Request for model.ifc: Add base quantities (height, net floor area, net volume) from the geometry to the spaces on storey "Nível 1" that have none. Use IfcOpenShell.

First a look at what the model holds.

```python
import ifcopenshell
import ifcopenshell.util.element
import ifcopenshell.util.unit

model = ifcopenshell.open("model.ifc")
print(model.schema)
for unit_type in ("LENGTHUNIT", "AREAUNIT", "VOLUMEUNIT"):
    print(unit_type, ifcopenshell.util.unit.calculate_unit_scale(model, unit_type))
storey = next(s for s in model.by_type("IfcBuildingStorey") if s.Name == "Nível 1")
spaces = [e for e in ifcopenshell.util.element.get_decomposition(storey) if e.is_a("IfcSpace")]
for e in sorted(spaces, key=lambda e: e.id()):
    print(e.id(), e.is_a(), e.Name, list(ifcopenshell.util.element.get_psets(e, qtos_only=True)), sep=" | ")
```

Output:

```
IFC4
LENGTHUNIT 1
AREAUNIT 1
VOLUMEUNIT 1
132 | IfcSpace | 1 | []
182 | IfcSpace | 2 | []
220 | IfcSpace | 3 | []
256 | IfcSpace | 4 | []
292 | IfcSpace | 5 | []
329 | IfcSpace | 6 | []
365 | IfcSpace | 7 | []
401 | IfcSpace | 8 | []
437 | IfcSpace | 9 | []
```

```python
import ifcopenshell
import ifcopenshell.api.pset
import ifcopenshell.geom
import ifcopenshell.util.element
import ifcopenshell.util.shape
import ifcopenshell.util.unit

model = ifcopenshell.open("model.ifc")
unit_scale = ifcopenshell.util.unit.calculate_unit_scale(model)
area_scale = ifcopenshell.util.unit.calculate_unit_scale(model, "AREAUNIT")
volume_scale = ifcopenshell.util.unit.calculate_unit_scale(model, "VOLUMEUNIT")
settings = ifcopenshell.geom.settings()

storey = next(s for s in model.by_type("IfcBuildingStorey") if s.Name == "Nível 1")
spaces = [e for e in ifcopenshell.util.element.get_decomposition(storey) if e.is_a("IfcSpace")]

for e in sorted(spaces, key=lambda e: e.id()):
    if ifcopenshell.util.element.get_psets(e, qtos_only=True, should_inherit=False):
        continue
    # Geometry comes back in metres, in the element's own axes.
    shape = ifcopenshell.geom.create_shape(settings, e)
    values = {
        "Height": ifcopenshell.util.shape.get_z(shape.geometry) / unit_scale,
        "NetFloorArea": ifcopenshell.util.shape.get_footprint_area(shape.geometry) / area_scale,
        "NetVolume": ifcopenshell.util.shape.get_volume(shape.geometry) / volume_scale,
    }
    qto = ifcopenshell.api.pset.add_qto(model, product=e, name="Qto_SpaceBaseQuantities")
    ifcopenshell.api.pset.edit_qto(model, qto=qto, properties=values)
    print(e.id(), {k: round(v, 3) for k, v in values.items()})

model.write("model_updated.ifc")
```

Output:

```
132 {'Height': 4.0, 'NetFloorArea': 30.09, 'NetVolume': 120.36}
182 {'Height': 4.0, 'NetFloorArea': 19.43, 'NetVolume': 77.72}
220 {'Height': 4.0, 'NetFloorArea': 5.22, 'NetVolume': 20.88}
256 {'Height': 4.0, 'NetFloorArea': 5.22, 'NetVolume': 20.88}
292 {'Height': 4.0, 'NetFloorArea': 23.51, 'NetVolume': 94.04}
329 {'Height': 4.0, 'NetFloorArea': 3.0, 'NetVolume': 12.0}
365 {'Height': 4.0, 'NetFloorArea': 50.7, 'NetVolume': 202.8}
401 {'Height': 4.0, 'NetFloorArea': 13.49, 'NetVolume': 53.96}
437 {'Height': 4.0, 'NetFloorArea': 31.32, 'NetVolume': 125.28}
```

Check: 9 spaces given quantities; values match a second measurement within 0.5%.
